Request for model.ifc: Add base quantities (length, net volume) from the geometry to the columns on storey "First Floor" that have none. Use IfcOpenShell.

First a look at what the model holds.

```python
import ifcopenshell
import ifcopenshell.util.element
import ifcopenshell.util.unit

model = ifcopenshell.open("model.ifc")
print(model.schema)
for unit_type in ("LENGTHUNIT", "AREAUNIT", "VOLUMEUNIT"):
    print(unit_type, ifcopenshell.util.unit.calculate_unit_scale(model, unit_type))
storey = next(s for s in model.by_type("IfcBuildingStorey") if s.Name == "First Floor")
columns = [e for e in ifcopenshell.util.element.get_decomposition(storey) if e.is_a("IfcColumn")]
for e in sorted(columns, key=lambda e: e.id()):
    print(e.id(), e.is_a(), e.Name, list(ifcopenshell.util.element.get_psets(e, qtos_only=True)), sep=" | ")
```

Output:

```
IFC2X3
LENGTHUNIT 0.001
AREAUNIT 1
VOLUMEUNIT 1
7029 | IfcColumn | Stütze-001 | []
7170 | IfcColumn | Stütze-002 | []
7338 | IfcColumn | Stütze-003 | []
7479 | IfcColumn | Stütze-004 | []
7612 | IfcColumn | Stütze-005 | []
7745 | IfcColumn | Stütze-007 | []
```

```python
import ifcopenshell
import ifcopenshell.api.pset
import ifcopenshell.geom
import ifcopenshell.util.element
import ifcopenshell.util.shape
import ifcopenshell.util.unit

model = ifcopenshell.open("model.ifc")
unit_scale = ifcopenshell.util.unit.calculate_unit_scale(model)
volume_scale = ifcopenshell.util.unit.calculate_unit_scale(model, "VOLUMEUNIT")
settings = ifcopenshell.geom.settings()

storey = next(s for s in model.by_type("IfcBuildingStorey") if s.Name == "First Floor")
columns = [e for e in ifcopenshell.util.element.get_decomposition(storey) if e.is_a("IfcColumn")]

for e in sorted(columns, key=lambda e: e.id()):
    if ifcopenshell.util.element.get_psets(e, qtos_only=True, should_inherit=False):
        continue
    # Geometry comes back in metres, in the element's own axes.
    shape = ifcopenshell.geom.create_shape(settings, e)
    values = {
        "Length": ifcopenshell.util.shape.get_z(shape.geometry) / unit_scale,
        "NetVolume": ifcopenshell.util.shape.get_volume(shape.geometry) / volume_scale,
    }
    qto = ifcopenshell.api.pset.add_qto(model, product=e, name="BaseQuantities")
    ifcopenshell.api.pset.edit_qto(model, qto=qto, properties=values)
    print(e.id(), {k: round(v, 3) for k, v in values.items()})

model.write("model_rev.ifc")
```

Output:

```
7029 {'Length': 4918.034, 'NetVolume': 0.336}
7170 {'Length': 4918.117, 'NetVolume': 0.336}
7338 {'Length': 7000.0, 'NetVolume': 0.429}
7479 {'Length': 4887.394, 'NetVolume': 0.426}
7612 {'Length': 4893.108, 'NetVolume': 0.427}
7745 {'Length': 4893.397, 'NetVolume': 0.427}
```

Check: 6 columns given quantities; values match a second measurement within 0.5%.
